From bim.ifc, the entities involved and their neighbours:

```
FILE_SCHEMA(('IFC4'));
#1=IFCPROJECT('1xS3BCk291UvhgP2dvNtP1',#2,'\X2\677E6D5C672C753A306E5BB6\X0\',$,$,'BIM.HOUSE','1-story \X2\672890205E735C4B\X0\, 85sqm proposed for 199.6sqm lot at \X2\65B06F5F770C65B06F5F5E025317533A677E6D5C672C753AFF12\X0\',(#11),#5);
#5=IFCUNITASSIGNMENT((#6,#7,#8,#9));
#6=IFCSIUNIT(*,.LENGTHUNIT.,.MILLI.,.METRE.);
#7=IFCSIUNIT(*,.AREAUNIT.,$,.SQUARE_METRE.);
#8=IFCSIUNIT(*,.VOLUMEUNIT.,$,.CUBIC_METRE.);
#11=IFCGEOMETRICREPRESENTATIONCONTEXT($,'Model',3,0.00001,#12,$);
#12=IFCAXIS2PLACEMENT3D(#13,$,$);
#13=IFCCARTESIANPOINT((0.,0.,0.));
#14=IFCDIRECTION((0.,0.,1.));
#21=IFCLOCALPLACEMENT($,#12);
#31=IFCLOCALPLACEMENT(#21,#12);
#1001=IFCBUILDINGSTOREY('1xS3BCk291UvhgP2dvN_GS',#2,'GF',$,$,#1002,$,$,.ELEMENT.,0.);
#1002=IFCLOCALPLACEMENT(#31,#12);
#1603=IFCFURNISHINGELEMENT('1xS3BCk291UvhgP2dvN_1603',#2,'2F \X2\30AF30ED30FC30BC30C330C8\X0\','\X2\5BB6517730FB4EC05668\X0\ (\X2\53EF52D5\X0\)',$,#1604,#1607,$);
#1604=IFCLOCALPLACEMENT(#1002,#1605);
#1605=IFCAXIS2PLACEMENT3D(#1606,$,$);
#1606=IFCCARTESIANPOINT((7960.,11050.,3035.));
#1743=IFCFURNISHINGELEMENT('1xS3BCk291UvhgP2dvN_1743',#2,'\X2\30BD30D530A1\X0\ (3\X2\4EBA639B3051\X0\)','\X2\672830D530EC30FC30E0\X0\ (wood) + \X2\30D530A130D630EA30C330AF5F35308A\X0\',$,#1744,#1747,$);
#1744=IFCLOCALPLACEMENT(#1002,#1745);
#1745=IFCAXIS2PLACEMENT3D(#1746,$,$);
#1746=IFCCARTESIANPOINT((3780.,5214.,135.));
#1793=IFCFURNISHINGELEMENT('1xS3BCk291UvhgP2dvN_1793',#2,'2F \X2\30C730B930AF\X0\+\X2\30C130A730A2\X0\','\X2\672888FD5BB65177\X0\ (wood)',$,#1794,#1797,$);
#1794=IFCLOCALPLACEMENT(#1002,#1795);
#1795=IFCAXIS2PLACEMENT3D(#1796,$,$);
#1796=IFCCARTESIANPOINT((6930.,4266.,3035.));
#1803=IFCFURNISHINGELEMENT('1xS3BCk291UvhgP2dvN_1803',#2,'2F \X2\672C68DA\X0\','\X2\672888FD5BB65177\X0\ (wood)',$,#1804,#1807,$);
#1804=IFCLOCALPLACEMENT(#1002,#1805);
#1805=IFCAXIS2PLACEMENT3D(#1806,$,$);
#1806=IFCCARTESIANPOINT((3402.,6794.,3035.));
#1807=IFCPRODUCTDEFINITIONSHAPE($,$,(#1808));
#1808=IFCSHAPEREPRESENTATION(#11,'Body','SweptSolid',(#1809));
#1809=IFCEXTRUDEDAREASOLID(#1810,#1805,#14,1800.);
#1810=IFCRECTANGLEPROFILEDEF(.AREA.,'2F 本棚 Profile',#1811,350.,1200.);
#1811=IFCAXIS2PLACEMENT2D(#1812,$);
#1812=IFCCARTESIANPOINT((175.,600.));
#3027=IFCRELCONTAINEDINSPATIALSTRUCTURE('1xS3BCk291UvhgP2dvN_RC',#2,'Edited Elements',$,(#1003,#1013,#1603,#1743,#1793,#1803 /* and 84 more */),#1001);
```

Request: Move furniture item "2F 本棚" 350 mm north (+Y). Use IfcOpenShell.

```python
import ifcopenshell
import ifcopenshell.api.geometry
import ifcopenshell.util.placement
import ifcopenshell.util.unit

model = ifcopenshell.open("bim.ifc")
unit_scale = ifcopenshell.util.unit.calculate_unit_scale(model)

item = model.by_guid("1xS3BCk291UvhgP2dvN_1803")
matrix = ifcopenshell.util.placement.get_local_placement(item.ObjectPlacement)
matrix[1, 3] += 0.35 / unit_scale
ifcopenshell.api.geometry.edit_object_placement(model, product=item, matrix=matrix, is_si=False)

print(ifcopenshell.util.placement.get_local_placement(item.ObjectPlacement).round(3) + 0.0)

model.write("bim_rev.ifc")
```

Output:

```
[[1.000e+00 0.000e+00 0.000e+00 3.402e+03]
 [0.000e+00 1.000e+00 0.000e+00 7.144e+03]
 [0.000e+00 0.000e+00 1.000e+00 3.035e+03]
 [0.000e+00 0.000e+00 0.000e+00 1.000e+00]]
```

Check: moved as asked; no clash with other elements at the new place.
